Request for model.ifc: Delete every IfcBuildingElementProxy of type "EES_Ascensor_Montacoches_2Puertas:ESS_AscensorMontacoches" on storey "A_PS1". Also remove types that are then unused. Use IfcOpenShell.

First a look at what the model holds.

```python
import ifcopenshell
import ifcopenshell.util.element

model = ifcopenshell.open("model.ifc")
print(model.schema)
storey = next(s for s in model.by_type("IfcBuildingStorey") if s.Name == "A_PS1")
proxies = [e for e in ifcopenshell.util.element.get_decomposition(storey) if e.is_a("IfcBuildingElementProxy")]
seen = {}
for e in proxies:
    element_type = ifcopenshell.util.element.get_type(e)
    name = element_type.Name if element_type not in (None, e) else None
    seen[name] = seen.get(name, 0) + 1
for name, count in sorted(seen.items(), key=str):
    print(count, "x", name)
```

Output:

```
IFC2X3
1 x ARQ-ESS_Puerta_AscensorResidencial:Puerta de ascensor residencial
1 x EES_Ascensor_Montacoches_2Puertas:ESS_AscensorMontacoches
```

```python
import ifcopenshell
import ifcopenshell.api.root
import ifcopenshell.util.element

model = ifcopenshell.open("model.ifc")

storey = next(s for s in model.by_type("IfcBuildingStorey") if s.Name == "A_PS1")
proxies = [e for e in ifcopenshell.util.element.get_decomposition(storey) if e.is_a("IfcBuildingElementProxy")]
targets = [e for e in proxies if (t := ifcopenshell.util.element.get_type(e)) not in (None, e) and t.Name == "EES_Ascensor_Montacoches_2Puertas:ESS_AscensorMontacoches"]
types = {ifcopenshell.util.element.get_type(e) for e in targets} - {None, *targets}

for e in targets:
    ifcopenshell.api.root.remove_product(model, product=e)
print(len(targets), "removed")

unused = [t for t in types if not ifcopenshell.util.element.get_types(t)]
for t in unused:
    ifcopenshell.api.root.remove_product(model, product=t)
print(len(unused), "unused types removed")

model.write("model_edited.ifc")
```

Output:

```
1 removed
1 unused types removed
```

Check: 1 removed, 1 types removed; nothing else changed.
